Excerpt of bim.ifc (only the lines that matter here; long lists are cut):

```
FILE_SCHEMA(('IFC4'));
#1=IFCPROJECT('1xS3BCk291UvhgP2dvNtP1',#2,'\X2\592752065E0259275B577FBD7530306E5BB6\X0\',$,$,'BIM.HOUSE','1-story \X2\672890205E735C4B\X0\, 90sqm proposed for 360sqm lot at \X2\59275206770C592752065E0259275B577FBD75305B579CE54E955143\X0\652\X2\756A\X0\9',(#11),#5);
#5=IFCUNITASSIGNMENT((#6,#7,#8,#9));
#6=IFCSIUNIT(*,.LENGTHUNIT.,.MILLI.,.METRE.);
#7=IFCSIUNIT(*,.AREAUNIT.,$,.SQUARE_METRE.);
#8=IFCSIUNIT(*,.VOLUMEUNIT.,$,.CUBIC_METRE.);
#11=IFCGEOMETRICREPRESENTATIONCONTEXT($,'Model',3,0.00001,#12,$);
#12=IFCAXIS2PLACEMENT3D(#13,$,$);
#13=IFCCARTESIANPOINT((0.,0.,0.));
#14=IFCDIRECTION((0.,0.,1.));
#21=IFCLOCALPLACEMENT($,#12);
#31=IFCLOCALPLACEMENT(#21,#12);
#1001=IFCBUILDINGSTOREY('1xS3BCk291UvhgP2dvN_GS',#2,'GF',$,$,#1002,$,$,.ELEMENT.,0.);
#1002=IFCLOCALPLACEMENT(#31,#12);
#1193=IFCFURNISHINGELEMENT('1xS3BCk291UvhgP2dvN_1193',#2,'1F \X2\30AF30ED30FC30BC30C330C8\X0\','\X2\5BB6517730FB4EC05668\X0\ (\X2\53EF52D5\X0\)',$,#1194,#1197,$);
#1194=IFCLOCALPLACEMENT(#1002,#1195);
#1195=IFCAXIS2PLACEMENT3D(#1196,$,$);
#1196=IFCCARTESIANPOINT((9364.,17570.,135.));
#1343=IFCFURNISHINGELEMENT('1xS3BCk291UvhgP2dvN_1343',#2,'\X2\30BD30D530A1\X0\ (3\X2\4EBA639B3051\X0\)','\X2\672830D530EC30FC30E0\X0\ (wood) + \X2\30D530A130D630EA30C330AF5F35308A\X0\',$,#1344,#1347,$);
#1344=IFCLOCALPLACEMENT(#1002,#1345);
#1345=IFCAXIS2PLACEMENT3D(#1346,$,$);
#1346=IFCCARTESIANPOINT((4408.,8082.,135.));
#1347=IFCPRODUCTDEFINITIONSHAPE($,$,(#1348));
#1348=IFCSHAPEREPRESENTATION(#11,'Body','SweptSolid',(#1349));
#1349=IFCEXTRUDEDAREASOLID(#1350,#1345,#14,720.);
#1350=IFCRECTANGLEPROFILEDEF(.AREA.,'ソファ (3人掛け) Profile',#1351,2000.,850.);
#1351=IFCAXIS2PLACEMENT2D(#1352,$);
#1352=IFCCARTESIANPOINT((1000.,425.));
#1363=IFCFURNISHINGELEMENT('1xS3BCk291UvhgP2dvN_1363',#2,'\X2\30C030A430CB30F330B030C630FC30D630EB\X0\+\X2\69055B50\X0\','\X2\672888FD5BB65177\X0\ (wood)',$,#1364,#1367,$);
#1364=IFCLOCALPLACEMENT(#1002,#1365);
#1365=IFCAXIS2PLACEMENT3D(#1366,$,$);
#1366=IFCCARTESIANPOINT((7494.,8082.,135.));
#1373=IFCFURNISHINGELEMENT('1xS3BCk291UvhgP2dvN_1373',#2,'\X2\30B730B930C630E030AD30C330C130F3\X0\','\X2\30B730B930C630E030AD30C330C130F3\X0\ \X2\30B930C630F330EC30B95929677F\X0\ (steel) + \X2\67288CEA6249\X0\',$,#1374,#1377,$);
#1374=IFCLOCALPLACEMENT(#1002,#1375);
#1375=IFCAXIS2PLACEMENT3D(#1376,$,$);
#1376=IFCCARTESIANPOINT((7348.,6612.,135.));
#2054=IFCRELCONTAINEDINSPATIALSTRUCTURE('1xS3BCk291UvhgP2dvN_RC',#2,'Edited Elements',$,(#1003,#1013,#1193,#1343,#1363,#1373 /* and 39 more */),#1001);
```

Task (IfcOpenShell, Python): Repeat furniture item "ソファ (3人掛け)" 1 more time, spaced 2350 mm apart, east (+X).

```python
import numpy as np
import ifcopenshell
import ifcopenshell.api.geometry
import ifcopenshell.api.root
import ifcopenshell.util.element
import ifcopenshell.util.placement

model = ifcopenshell.open("bim.ifc")


def reuse_history(source, copy):
    """copy_class also copies each property set's owner history, people and application; keep the originals."""
    for rel in copy.IsDefinedBy:
        if rel.is_a("IfcRelDefinesByProperties") and (history := rel.RelatingPropertyDefinition.OwnerHistory):
            rel.RelatingPropertyDefinition.OwnerHistory = source.OwnerHistory
            ifcopenshell.util.element.remove_deep2(model, history)


source = model.by_id(1343)
base = ifcopenshell.util.placement.get_local_placement(source.ObjectPlacement)
step = np.array([1.0, 0.0, 0.0]) * 2350.0

for i in range(1, 2):
    copy = ifcopenshell.api.root.copy_class(model, product=source)
    copy.Representation = ifcopenshell.util.element.copy_deep(
        model, source.Representation, exclude=["IfcGeometricRepresentationContext", "IfcRepresentationMap"]
    )
    reuse_history(source, copy)
    matrix = base.copy()
    matrix[:3, 3] += i * step
    print("added at", matrix[:3, 3].round(3) + 0.0)
    ifcopenshell.api.geometry.edit_object_placement(model, product=copy, matrix=matrix, is_si=False)

model.write("bim-out.ifc")
```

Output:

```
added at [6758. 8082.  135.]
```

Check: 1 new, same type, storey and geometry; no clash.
